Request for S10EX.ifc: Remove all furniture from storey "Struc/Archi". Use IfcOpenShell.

First a look at what the model holds.

```python
import ifcopenshell
import ifcopenshell.util.element

model = ifcopenshell.open("S10EX.ifc")
print(model.schema)
storey = next(s for s in model.by_type("IfcBuildingStorey") if s.Name == "Struc/Archi")
furniture = [e for e in ifcopenshell.util.element.get_decomposition(storey) if e.is_a("IfcFurnishingElement")]
seen = {}
for e in furniture:
    element_type = ifcopenshell.util.element.get_type(e)
    name = element_type.Name if element_type not in (None, e) else None
    seen[name] = seen.get(name, 0) + 1
for name, count in sorted(seen.items(), key=str):
    print(count, "x", name)
```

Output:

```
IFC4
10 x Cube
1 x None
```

```python
import ifcopenshell
import ifcopenshell.api.root
import ifcopenshell.util.element

model = ifcopenshell.open("S10EX.ifc")

storey = next(s for s in model.by_type("IfcBuildingStorey") if s.Name == "Struc/Archi")
furniture = [e for e in ifcopenshell.util.element.get_decomposition(storey) if e.is_a("IfcFurnishingElement")]

for e in furniture:
    ifcopenshell.api.root.remove_product(model, product=e)
print(len(furniture), "removed")

model.write("S10EX_updated.ifc")
```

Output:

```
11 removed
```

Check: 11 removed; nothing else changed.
